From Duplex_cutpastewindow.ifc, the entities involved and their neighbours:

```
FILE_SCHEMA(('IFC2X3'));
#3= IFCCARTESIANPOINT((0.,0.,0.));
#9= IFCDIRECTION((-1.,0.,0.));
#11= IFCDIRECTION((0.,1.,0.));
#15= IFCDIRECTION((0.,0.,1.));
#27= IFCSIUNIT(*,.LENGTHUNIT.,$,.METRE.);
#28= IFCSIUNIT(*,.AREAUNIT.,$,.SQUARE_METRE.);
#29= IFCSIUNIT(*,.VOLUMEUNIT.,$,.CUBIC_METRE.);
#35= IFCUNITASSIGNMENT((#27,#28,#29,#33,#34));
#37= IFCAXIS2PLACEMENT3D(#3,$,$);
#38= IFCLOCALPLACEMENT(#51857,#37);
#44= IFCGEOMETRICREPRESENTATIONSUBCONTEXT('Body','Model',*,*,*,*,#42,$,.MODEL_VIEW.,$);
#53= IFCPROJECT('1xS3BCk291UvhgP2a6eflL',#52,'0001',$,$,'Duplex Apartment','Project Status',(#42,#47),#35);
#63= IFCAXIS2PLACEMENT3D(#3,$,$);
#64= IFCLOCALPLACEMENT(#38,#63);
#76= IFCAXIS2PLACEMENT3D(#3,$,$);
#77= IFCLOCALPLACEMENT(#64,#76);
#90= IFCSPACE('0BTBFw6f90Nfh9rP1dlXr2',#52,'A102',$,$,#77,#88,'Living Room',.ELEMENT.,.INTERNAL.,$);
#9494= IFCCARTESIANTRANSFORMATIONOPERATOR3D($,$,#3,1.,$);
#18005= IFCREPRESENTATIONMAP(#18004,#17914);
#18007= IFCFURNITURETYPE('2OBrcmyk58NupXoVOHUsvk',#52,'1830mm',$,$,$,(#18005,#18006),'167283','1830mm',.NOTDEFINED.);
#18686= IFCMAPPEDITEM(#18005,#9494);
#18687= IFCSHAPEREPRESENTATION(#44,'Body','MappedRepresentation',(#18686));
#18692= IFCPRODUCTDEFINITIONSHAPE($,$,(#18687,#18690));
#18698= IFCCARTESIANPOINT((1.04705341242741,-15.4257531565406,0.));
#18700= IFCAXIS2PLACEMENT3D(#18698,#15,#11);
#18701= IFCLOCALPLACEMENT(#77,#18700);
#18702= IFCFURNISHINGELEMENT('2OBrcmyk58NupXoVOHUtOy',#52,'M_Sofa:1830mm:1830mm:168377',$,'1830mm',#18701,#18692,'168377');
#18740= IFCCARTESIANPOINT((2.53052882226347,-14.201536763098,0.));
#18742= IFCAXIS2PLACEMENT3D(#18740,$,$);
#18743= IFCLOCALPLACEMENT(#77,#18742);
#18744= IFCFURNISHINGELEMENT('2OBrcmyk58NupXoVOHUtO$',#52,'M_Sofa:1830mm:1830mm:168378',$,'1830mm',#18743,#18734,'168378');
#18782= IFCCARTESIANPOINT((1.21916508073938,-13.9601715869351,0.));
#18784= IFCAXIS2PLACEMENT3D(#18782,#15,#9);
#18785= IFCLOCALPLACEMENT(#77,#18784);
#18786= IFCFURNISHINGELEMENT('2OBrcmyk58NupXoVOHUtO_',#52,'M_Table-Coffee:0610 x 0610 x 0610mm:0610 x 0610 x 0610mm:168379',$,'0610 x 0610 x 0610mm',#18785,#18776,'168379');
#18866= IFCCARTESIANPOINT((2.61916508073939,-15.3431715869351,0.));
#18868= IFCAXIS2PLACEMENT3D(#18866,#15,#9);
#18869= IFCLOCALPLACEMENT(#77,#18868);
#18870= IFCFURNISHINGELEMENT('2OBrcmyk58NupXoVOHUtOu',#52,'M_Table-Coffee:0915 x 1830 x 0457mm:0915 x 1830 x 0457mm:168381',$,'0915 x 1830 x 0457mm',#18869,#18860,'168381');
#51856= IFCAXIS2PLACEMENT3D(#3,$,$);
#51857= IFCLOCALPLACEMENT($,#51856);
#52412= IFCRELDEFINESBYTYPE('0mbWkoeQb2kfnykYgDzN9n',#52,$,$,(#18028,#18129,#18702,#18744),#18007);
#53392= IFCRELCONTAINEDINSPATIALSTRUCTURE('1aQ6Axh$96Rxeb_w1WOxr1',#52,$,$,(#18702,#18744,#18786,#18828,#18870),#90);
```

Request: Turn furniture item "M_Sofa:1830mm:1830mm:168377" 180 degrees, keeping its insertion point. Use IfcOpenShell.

```python
import ifcopenshell
import ifcopenshell.api.geometry
import ifcopenshell.util.placement

model = ifcopenshell.open("Duplex_cutpastewindow.ifc")

item = model.by_guid("2OBrcmyk58NupXoVOHUtOy")
matrix = ifcopenshell.util.placement.get_local_placement(item.ObjectPlacement)
matrix = matrix @ ifcopenshell.util.placement.rotation(180, "Z")
ifcopenshell.api.geometry.edit_object_placement(model, product=item, matrix=matrix, is_si=False)

print(ifcopenshell.util.placement.get_local_placement(item.ObjectPlacement).round(3) + 0.0)

model.write("Duplex_cutpastewindow-out.ifc")
```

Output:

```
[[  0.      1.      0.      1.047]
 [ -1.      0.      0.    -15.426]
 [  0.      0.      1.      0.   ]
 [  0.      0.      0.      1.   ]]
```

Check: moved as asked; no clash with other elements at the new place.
